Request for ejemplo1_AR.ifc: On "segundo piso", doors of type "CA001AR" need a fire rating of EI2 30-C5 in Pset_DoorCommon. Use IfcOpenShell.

First a look at what the model holds.

```python
import ifcopenshell
import ifcopenshell.util.element

model = ifcopenshell.open("ejemplo1_AR.ifc")
print(model.schema)
storey = next(s for s in model.by_type("IfcBuildingStorey") if s.Name == "segundo piso")
doors = [e for e in ifcopenshell.util.element.get_decomposition(storey) if e.is_a("IfcDoor")]
seen = {}
for e in doors:
    element_type = ifcopenshell.util.element.get_type(e)
    key = (element_type.Name if element_type != e and element_type else None, ifcopenshell.util.element.get_pset(e, "Pset_DoorCommon", "FireRating"))
    seen[key] = seen.get(key, 0) + 1
for (name, value), count in sorted(seen.items(), key=str):
    print(count, "x", name, "|", value)
```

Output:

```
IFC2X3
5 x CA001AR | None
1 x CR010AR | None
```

```python
import ifcopenshell
import ifcopenshell.api.pset
import ifcopenshell.util.element

model = ifcopenshell.open("ejemplo1_AR.ifc")

storey = next(s for s in model.by_type("IfcBuildingStorey") if s.Name == "segundo piso")
doors = [e for e in ifcopenshell.util.element.get_decomposition(storey) if e.is_a("IfcDoor")]

count = 0
for e in doors:
    element_type = ifcopenshell.util.element.get_type(e)
    if element_type in (None, e) or element_type.Name != "CA001AR":
        continue
    # add_pset returns the element's existing set when there is one.
    pset = ifcopenshell.api.pset.add_pset(model, product=e, name="Pset_DoorCommon")
    ifcopenshell.api.pset.edit_pset(model, pset=pset, properties={"FireRating": "EI2 30-C5"})
    count += 1

print(count, "doors updated")

model.write("ejemplo1_AR_edited.ifc")
```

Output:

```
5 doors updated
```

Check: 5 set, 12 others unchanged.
